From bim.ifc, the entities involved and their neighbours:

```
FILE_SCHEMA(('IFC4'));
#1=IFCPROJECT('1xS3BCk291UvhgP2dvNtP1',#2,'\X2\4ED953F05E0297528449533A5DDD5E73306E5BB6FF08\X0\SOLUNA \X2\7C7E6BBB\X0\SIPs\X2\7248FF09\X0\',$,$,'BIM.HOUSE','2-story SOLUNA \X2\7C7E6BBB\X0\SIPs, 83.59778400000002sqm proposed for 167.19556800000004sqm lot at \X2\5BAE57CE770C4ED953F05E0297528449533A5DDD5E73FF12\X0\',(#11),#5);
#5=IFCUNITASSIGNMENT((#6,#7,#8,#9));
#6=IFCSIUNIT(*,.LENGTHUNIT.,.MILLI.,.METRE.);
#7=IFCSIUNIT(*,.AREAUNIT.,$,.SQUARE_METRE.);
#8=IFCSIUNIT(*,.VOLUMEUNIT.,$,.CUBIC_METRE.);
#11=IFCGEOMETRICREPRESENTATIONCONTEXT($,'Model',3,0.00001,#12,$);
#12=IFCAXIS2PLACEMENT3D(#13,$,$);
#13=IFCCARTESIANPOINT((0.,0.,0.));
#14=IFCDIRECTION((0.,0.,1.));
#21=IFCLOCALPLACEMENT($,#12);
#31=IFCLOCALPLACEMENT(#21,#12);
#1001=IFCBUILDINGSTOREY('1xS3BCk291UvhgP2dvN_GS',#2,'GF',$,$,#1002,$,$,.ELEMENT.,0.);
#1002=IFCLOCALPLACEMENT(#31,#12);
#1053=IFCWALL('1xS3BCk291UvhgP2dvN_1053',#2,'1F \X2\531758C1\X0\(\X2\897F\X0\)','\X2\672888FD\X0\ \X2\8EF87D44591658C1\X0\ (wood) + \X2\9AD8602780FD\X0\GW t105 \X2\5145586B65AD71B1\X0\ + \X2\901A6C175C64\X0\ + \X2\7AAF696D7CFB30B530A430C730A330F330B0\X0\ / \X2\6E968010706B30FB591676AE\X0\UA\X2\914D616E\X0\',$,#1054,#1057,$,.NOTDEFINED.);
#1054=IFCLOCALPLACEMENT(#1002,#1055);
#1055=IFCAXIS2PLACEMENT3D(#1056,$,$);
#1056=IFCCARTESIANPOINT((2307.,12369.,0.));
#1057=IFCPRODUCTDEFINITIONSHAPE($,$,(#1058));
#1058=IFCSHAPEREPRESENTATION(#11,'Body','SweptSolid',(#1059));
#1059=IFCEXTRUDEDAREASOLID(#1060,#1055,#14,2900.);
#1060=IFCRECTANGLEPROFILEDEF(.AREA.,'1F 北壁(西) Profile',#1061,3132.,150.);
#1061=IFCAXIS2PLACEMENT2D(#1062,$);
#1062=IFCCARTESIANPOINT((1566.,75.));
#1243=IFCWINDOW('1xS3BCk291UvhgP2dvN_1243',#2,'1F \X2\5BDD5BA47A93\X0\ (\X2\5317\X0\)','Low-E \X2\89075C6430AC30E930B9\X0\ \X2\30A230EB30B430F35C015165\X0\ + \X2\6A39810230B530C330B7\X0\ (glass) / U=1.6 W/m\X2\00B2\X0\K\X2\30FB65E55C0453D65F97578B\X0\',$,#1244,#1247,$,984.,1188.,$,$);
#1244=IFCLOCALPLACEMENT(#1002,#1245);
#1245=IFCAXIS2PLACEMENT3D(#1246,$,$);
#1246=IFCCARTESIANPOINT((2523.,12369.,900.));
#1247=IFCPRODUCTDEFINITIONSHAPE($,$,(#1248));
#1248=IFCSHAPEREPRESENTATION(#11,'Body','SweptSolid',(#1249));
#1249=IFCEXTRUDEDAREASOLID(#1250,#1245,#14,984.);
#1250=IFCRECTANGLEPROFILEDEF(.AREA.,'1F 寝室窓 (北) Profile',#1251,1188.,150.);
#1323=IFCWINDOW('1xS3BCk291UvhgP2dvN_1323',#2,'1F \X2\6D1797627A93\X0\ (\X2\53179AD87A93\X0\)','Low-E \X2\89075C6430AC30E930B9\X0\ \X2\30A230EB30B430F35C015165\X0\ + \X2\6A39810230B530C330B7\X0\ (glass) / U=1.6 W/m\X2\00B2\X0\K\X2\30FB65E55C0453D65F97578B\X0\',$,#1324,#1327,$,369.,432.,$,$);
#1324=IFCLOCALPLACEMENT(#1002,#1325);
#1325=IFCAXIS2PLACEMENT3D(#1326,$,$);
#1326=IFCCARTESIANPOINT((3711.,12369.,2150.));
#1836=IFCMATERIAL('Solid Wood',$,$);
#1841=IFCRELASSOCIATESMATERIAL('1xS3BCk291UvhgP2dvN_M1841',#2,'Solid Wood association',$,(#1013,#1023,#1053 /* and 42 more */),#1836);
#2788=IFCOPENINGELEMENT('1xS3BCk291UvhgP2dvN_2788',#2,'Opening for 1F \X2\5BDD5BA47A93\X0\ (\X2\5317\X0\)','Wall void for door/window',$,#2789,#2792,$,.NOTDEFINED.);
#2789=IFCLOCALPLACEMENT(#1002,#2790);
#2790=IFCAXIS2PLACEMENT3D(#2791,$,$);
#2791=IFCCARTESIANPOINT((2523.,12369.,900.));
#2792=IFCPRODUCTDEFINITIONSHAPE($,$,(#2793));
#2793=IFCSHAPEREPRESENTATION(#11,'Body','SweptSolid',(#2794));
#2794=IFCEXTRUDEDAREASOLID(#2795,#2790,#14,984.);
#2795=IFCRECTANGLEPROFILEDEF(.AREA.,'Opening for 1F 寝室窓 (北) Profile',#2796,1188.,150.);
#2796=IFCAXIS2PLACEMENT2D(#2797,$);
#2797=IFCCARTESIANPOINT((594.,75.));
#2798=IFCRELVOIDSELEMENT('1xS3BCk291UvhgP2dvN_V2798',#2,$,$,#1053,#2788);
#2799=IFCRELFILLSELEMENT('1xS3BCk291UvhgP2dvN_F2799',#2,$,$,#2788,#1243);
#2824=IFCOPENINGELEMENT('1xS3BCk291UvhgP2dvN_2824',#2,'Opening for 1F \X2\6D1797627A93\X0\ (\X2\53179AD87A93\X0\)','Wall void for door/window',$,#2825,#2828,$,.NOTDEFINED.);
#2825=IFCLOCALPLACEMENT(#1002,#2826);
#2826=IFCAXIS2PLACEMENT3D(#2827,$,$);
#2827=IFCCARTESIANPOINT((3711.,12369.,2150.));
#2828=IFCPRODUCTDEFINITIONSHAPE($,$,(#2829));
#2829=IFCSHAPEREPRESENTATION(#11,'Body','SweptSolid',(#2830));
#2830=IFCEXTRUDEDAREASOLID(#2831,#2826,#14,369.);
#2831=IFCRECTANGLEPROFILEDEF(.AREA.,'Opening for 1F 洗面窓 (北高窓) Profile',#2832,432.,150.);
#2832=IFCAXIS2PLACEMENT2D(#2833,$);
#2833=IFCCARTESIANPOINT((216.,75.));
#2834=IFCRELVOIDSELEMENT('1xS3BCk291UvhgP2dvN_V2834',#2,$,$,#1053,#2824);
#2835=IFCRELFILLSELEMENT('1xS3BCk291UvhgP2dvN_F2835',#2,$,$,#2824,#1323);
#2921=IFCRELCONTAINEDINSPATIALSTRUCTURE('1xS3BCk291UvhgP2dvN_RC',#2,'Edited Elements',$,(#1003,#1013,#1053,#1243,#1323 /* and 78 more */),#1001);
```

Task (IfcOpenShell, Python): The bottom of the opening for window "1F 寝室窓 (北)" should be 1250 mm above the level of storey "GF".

```python
import numpy as np
import ifcopenshell
import ifcopenshell.api.geometry
import ifcopenshell.geom
import ifcopenshell.util.element
import ifcopenshell.util.placement
import ifcopenshell.util.shape
import ifcopenshell.util.unit

model = ifcopenshell.open("bim.ifc")
unit_scale = ifcopenshell.util.unit.calculate_unit_scale(model)

window = model.by_guid("1xS3BCk291UvhgP2dvN_1243")
opening = window.FillsVoids[0].RelatingOpeningElement
storey = ifcopenshell.util.element.get_container(window, ifc_class="IfcBuildingStorey")
level = ifcopenshell.util.placement.get_local_placement(storey.ObjectPlacement)[2, 3]

# The opening's origin need not be at the sill, so measure its lowest point.
shape = ifcopenshell.geom.create_shape(ifcopenshell.geom.settings(), opening)
bottom = ifcopenshell.util.shape.get_shape_bottom_elevation(shape, shape.geometry) / unit_scale
dz = level + 1.25 / unit_scale - bottom

shift = np.array([0.0, 0.0, dz])
# The window is not placed relative to its opening, so move both.
for product in (opening, window):
    matrix = ifcopenshell.util.placement.get_local_placement(product.ObjectPlacement)
    matrix[:3, 3] += shift
    ifcopenshell.api.geometry.edit_object_placement(model, product=product, matrix=matrix, is_si=False)

print(f"moved by {dz * unit_scale:+.3f} m")

model.write("bim_updated.ifc")
```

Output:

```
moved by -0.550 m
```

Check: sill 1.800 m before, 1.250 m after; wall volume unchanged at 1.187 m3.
